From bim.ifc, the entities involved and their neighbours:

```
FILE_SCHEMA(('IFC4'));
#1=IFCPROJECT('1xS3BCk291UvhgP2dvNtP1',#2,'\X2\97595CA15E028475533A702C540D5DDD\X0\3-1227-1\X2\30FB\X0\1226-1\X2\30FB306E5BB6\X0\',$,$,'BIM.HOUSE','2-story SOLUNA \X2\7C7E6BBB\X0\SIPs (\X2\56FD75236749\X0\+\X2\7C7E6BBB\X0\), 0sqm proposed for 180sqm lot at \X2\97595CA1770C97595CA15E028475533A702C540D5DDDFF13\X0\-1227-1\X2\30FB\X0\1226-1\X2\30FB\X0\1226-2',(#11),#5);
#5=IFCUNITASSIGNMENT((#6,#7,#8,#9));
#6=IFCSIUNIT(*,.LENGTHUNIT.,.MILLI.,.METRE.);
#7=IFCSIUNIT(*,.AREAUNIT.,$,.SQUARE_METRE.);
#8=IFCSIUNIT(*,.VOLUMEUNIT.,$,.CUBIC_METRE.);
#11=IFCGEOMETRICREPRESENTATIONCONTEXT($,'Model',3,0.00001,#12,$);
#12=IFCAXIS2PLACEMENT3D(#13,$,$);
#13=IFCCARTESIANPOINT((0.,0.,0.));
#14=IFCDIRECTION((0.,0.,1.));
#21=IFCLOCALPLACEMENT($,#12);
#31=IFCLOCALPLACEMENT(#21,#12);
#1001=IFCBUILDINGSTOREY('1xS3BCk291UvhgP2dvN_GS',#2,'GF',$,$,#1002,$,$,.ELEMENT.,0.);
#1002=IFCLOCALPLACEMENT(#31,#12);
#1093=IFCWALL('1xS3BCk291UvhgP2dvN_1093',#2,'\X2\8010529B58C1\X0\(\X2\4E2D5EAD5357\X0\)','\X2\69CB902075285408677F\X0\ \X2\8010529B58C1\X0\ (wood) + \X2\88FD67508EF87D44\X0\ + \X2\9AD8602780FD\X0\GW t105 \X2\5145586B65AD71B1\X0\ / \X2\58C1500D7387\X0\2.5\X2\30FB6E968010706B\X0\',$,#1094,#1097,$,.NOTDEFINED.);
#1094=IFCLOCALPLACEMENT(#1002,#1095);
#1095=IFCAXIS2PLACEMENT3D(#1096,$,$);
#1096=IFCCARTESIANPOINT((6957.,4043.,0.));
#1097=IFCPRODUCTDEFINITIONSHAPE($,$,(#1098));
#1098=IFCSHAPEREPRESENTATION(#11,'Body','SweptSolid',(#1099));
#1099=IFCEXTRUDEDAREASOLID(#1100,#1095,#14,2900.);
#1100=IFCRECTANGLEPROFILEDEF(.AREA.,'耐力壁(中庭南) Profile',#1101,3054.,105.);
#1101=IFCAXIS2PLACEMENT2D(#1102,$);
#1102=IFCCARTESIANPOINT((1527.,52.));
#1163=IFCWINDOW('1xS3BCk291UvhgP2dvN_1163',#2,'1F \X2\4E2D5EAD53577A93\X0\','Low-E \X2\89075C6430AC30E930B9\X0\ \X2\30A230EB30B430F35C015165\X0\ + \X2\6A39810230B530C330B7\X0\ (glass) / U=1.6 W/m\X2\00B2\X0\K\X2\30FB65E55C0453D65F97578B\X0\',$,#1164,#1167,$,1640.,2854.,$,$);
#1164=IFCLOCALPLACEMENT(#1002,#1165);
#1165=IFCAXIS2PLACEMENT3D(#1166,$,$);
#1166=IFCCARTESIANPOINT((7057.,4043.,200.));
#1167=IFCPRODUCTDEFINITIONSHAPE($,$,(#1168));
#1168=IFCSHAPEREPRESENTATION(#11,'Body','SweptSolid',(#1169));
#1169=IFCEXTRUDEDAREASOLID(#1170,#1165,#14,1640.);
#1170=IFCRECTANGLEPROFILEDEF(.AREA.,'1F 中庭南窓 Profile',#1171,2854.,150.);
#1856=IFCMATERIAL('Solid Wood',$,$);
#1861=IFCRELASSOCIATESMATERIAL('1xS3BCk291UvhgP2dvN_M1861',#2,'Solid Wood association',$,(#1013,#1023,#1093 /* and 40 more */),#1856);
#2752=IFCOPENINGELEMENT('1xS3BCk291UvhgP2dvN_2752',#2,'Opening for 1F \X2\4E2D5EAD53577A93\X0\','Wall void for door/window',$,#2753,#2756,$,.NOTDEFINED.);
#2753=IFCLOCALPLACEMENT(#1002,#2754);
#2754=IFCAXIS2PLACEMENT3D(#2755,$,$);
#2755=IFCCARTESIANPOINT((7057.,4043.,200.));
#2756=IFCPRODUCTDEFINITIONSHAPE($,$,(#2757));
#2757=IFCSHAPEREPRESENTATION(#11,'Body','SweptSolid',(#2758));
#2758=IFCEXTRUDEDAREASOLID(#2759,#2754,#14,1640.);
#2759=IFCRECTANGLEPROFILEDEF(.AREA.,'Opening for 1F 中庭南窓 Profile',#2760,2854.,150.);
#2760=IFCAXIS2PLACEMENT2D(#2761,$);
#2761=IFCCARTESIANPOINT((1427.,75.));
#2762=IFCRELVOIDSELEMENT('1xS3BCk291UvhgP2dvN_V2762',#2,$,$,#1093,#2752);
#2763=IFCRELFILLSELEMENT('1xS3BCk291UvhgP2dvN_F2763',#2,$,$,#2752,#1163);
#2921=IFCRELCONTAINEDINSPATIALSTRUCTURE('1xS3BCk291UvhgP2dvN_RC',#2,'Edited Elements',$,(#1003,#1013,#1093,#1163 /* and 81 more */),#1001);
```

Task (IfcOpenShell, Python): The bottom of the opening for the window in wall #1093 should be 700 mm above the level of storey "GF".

```python
import numpy as np
import ifcopenshell
import ifcopenshell.api.geometry
import ifcopenshell.geom
import ifcopenshell.util.element
import ifcopenshell.util.placement
import ifcopenshell.util.shape
import ifcopenshell.util.unit

model = ifcopenshell.open("bim.ifc")
unit_scale = ifcopenshell.util.unit.calculate_unit_scale(model)

window = model.by_guid("1xS3BCk291UvhgP2dvN_1163")
opening = window.FillsVoids[0].RelatingOpeningElement
storey = ifcopenshell.util.element.get_container(window, ifc_class="IfcBuildingStorey")
level = ifcopenshell.util.placement.get_local_placement(storey.ObjectPlacement)[2, 3]

# The opening's origin need not be at the sill, so measure its lowest point.
shape = ifcopenshell.geom.create_shape(ifcopenshell.geom.settings(), opening)
bottom = ifcopenshell.util.shape.get_shape_bottom_elevation(shape, shape.geometry) / unit_scale
dz = level + 0.7 / unit_scale - bottom

shift = np.array([0.0, 0.0, dz])
# The window is not placed relative to its opening, so move both.
for product in (opening, window):
    matrix = ifcopenshell.util.placement.get_local_placement(product.ObjectPlacement)
    matrix[:3, 3] += shift
    ifcopenshell.api.geometry.edit_object_placement(model, product=product, matrix=matrix, is_si=False)

print(f"moved by {dz * unit_scale:+.3f} m")

model.write("bim_rev.ifc")
```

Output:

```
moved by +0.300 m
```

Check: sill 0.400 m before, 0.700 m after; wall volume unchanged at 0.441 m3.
